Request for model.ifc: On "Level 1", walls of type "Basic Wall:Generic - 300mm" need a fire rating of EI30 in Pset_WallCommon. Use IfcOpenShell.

First a look at what the model holds.

```python
import ifcopenshell
import ifcopenshell.util.element

model = ifcopenshell.open("model.ifc")
print(model.schema)
storey = next(s for s in model.by_type("IfcBuildingStorey") if s.Name == "Level 1")
walls = [e for e in ifcopenshell.util.element.get_decomposition(storey) if e.is_a("IfcWall")]
seen = {}
for e in walls:
    element_type = ifcopenshell.util.element.get_type(e)
    key = (element_type.Name if element_type != e and element_type else None, ifcopenshell.util.element.get_pset(e, "Pset_WallCommon", "FireRating"))
    seen[key] = seen.get(key, 0) + 1
for (name, value), count in sorted(seen.items(), key=str):
    print(count, "x", name, "|", value)
```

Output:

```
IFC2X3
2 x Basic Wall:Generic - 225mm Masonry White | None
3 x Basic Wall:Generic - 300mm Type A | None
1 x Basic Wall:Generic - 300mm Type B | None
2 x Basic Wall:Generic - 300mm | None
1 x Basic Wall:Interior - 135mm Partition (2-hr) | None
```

```python
import ifcopenshell
import ifcopenshell.api.pset
import ifcopenshell.util.element

model = ifcopenshell.open("model.ifc")

storey = next(s for s in model.by_type("IfcBuildingStorey") if s.Name == "Level 1")
walls = [e for e in ifcopenshell.util.element.get_decomposition(storey) if e.is_a("IfcWall")]

count = 0
for e in walls:
    element_type = ifcopenshell.util.element.get_type(e)
    if element_type in (None, e) or element_type.Name != "Basic Wall:Generic - 300mm":
        continue
    # add_pset returns the element's existing set when there is one.
    pset = ifcopenshell.api.pset.add_pset(model, product=e, name="Pset_WallCommon")
    ifcopenshell.api.pset.edit_pset(model, pset=pset, properties={"FireRating": "EI30"})
    count += 1

print(count, "walls updated")

model.write("model_edited.ifc")
```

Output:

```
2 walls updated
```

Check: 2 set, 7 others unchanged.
